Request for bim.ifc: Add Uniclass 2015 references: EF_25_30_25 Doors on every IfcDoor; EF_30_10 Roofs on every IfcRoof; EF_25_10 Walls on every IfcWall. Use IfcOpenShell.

First a look at what the model holds.

```python
import ifcopenshell

model = ifcopenshell.open("bim.ifc")
print(model.schema)
print("classifications:", [c.Name for c in model.by_type("IfcClassification")])
for ifc_class in ("IfcDoor", "IfcRoof", "IfcStair", "IfcWall", "IfcWindow"):
    print(ifc_class, len(model.by_type(ifc_class)))
```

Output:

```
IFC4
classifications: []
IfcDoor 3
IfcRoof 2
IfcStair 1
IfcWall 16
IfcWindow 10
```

```python
import ifcopenshell
import ifcopenshell.api.classification

model = ifcopenshell.open("bim.ifc")

system = ifcopenshell.api.classification.add_classification(model, classification="Uniclass 2015")

codes = {
    "IfcDoor": ("EF_25_30_25", "Doors"),
    "IfcRoof": ("EF_30_10", "Roofs"),
    "IfcWall": ("EF_25_10", "Walls"),
}
for ifc_class, (code, name) in codes.items():
    products = model.by_type(ifc_class)
    ifcopenshell.api.classification.add_reference(
        model, products=products, classification=system, identification=code, name=name
    )
    print(code, len(products))

model.write("bim_rev.ifc")
```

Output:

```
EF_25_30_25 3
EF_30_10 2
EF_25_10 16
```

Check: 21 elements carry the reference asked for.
